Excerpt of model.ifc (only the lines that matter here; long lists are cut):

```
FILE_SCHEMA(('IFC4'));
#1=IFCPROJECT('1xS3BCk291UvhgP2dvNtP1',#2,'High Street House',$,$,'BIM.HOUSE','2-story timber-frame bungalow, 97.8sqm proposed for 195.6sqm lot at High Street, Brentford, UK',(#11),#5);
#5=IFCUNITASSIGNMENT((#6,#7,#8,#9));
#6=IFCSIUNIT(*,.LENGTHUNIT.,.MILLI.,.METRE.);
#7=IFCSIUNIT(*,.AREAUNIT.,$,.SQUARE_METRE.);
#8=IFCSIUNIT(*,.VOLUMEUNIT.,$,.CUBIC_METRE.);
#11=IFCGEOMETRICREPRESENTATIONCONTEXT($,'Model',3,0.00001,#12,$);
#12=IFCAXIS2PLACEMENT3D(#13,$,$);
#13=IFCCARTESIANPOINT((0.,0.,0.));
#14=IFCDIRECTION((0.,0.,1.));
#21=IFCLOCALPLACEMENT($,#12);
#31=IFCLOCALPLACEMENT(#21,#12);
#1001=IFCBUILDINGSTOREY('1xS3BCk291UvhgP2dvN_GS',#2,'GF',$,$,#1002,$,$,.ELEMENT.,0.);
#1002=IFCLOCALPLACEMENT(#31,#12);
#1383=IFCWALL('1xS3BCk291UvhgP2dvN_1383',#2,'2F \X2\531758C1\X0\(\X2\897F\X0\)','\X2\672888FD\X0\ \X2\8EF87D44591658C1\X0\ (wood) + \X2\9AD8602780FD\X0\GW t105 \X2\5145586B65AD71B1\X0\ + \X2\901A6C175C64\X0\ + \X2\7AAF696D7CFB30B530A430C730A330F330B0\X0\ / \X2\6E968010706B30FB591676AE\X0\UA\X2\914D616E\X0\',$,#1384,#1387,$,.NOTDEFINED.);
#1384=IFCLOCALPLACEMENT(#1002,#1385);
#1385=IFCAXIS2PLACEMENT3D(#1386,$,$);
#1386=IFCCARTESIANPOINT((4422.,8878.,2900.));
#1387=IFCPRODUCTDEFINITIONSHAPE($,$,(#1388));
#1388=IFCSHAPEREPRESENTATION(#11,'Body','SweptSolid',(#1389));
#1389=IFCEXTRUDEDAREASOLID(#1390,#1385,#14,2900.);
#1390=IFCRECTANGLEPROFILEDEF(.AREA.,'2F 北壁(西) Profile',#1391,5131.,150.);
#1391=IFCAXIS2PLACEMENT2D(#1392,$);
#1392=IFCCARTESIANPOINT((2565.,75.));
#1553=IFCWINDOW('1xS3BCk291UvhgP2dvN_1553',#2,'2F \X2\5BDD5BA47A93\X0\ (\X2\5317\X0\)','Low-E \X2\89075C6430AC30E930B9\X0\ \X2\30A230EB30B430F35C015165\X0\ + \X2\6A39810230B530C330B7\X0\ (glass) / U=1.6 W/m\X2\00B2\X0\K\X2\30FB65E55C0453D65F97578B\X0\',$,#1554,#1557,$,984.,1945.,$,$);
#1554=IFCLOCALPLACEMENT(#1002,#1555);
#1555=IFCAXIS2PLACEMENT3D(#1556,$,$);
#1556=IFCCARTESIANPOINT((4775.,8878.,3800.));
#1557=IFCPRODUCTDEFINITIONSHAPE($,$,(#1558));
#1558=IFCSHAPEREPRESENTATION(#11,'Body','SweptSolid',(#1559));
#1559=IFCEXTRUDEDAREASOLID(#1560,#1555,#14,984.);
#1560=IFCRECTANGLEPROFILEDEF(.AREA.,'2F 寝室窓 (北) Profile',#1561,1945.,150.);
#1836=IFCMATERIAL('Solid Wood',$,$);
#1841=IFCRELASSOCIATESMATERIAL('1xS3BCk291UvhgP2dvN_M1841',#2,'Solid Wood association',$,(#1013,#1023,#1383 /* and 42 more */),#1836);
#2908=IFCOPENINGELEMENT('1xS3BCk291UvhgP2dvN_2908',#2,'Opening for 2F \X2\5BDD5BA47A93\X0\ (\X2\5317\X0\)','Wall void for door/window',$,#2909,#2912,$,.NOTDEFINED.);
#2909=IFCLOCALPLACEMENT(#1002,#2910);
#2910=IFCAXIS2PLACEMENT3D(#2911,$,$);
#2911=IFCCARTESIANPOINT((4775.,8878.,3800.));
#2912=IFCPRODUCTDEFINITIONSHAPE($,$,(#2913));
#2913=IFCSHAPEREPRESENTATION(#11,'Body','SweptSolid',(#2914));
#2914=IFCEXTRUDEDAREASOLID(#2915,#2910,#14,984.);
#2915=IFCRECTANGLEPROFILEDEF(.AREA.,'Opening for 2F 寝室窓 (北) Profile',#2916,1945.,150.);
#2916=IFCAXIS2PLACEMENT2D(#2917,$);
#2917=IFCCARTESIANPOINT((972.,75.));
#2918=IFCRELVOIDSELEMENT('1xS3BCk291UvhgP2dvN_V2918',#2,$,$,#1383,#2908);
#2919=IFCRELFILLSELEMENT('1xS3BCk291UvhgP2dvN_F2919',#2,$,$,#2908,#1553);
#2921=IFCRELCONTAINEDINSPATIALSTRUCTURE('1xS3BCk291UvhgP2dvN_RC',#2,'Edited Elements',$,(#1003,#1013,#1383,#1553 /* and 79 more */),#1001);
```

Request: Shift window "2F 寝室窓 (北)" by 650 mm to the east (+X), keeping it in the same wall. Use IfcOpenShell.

```python
import ifcopenshell
import ifcopenshell.api.geometry
import ifcopenshell.util.placement
import ifcopenshell.util.unit

model = ifcopenshell.open("model.ifc")
unit_scale = ifcopenshell.util.unit.calculate_unit_scale(model)

window = model.by_guid("1xS3BCk291UvhgP2dvN_1553")
opening = window.FillsVoids[0].RelatingOpeningElement
wall = opening.VoidsElements[0].RelatingBuildingElement

wall_matrix = ifcopenshell.util.placement.get_local_placement(wall.ObjectPlacement)
shift = wall_matrix[:3, 0] * 0.65 / unit_scale
before = ifcopenshell.util.placement.get_local_placement(window.ObjectPlacement)[:3, 3].copy()

# The window is not placed relative to its opening, so move both.
for product in (opening, window):
    matrix = ifcopenshell.util.placement.get_local_placement(product.ObjectPlacement)
    matrix[:3, 3] += shift
    ifcopenshell.api.geometry.edit_object_placement(model, product=product, matrix=matrix, is_si=False)

after = ifcopenshell.util.placement.get_local_placement(window.ObjectPlacement)[:3, 3]
print("window moved by", (after - before).round(3) + 0.0)

model.write("model_updated.ifc")
```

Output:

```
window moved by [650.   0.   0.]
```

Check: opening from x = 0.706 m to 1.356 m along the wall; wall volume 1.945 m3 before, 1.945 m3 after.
